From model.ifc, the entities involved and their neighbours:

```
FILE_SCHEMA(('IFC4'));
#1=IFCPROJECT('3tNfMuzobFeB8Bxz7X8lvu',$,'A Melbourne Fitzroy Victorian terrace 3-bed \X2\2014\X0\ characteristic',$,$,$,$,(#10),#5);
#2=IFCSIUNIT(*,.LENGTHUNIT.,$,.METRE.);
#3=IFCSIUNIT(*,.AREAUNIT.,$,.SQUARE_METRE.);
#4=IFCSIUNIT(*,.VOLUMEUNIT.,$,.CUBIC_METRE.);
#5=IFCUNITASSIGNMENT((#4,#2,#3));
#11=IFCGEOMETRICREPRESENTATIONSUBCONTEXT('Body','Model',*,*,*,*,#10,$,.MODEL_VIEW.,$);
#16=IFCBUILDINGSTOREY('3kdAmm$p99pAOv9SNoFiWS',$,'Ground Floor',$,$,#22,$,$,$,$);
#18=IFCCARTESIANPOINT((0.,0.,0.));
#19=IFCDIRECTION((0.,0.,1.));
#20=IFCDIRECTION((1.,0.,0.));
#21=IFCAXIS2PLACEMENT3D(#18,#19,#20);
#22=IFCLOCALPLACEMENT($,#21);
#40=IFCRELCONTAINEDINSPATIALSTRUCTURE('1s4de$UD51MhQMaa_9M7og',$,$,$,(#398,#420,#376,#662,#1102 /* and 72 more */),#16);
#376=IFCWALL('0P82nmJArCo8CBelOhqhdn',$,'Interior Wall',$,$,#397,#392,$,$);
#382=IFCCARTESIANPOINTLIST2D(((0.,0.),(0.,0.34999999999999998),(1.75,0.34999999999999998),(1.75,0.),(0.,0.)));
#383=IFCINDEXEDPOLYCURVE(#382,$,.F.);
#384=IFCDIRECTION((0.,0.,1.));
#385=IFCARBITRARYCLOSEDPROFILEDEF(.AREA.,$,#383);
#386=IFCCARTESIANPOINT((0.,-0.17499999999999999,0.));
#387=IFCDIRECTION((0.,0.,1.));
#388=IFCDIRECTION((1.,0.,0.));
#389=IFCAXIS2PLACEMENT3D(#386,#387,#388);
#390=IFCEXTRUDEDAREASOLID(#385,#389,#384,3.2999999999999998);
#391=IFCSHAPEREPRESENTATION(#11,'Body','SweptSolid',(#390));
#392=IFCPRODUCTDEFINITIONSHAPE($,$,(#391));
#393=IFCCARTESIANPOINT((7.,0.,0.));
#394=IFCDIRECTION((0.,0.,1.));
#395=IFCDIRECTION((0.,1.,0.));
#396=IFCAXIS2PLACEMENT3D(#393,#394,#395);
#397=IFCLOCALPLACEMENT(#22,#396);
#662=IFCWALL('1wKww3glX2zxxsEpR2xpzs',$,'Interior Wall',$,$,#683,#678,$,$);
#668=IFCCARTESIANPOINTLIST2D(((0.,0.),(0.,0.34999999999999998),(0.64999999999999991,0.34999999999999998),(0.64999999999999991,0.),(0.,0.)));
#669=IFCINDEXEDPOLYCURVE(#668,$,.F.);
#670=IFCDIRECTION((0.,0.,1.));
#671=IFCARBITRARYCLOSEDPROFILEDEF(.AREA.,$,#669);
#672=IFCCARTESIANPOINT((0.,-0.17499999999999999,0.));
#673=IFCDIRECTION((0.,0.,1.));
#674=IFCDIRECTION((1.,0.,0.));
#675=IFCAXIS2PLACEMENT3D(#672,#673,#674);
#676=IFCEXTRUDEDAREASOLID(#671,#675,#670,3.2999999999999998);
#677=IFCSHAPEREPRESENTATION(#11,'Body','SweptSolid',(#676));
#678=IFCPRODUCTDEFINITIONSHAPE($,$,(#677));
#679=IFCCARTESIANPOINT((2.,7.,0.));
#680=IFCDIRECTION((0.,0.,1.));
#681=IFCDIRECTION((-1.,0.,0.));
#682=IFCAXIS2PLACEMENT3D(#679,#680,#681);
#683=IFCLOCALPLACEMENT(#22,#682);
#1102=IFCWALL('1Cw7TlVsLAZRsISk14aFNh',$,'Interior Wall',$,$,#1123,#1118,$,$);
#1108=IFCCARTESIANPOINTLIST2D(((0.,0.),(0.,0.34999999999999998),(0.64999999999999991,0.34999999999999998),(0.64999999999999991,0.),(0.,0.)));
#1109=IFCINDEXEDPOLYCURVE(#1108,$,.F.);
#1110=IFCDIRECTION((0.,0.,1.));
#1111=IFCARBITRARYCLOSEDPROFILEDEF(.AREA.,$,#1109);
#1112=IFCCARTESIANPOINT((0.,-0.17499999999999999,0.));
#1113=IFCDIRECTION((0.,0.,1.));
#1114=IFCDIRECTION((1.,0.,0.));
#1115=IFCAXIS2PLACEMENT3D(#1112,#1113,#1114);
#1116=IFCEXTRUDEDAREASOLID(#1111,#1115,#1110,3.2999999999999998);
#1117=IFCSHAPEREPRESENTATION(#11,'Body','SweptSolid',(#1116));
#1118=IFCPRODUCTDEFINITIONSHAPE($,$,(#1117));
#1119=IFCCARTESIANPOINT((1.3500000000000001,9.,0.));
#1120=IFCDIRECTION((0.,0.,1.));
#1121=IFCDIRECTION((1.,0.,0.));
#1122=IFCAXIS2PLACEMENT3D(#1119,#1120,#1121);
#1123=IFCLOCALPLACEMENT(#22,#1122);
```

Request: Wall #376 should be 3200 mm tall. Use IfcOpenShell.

```python
import ifcopenshell
import ifcopenshell.geom
import ifcopenshell.util.representation
import ifcopenshell.util.shape
import ifcopenshell.util.unit

model = ifcopenshell.open("model.ifc")
unit_scale = ifcopenshell.util.unit.calculate_unit_scale(model)
settings = ifcopenshell.geom.settings()


def volume(element):
    """Net volume in cubic metres, openings subtracted."""
    shape = ifcopenshell.geom.create_shape(settings, element)
    return ifcopenshell.util.shape.get_volume(shape.geometry)


wall = model.by_id(376)
before = volume(wall)

body = ifcopenshell.util.representation.get_representation(wall, "Model", "Body")
solid = body.Items[0]
old_height = solid.Depth
solid.Depth = 3.2 / unit_scale
after = volume(wall)

print(f"height {old_height:g} -> {solid.Depth:g}, volume {before:.3f} -> {after:.3f} m3")

model.write("model_v2.ifc")
```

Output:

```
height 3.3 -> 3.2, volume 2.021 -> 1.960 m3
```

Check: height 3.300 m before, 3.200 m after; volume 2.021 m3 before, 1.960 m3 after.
